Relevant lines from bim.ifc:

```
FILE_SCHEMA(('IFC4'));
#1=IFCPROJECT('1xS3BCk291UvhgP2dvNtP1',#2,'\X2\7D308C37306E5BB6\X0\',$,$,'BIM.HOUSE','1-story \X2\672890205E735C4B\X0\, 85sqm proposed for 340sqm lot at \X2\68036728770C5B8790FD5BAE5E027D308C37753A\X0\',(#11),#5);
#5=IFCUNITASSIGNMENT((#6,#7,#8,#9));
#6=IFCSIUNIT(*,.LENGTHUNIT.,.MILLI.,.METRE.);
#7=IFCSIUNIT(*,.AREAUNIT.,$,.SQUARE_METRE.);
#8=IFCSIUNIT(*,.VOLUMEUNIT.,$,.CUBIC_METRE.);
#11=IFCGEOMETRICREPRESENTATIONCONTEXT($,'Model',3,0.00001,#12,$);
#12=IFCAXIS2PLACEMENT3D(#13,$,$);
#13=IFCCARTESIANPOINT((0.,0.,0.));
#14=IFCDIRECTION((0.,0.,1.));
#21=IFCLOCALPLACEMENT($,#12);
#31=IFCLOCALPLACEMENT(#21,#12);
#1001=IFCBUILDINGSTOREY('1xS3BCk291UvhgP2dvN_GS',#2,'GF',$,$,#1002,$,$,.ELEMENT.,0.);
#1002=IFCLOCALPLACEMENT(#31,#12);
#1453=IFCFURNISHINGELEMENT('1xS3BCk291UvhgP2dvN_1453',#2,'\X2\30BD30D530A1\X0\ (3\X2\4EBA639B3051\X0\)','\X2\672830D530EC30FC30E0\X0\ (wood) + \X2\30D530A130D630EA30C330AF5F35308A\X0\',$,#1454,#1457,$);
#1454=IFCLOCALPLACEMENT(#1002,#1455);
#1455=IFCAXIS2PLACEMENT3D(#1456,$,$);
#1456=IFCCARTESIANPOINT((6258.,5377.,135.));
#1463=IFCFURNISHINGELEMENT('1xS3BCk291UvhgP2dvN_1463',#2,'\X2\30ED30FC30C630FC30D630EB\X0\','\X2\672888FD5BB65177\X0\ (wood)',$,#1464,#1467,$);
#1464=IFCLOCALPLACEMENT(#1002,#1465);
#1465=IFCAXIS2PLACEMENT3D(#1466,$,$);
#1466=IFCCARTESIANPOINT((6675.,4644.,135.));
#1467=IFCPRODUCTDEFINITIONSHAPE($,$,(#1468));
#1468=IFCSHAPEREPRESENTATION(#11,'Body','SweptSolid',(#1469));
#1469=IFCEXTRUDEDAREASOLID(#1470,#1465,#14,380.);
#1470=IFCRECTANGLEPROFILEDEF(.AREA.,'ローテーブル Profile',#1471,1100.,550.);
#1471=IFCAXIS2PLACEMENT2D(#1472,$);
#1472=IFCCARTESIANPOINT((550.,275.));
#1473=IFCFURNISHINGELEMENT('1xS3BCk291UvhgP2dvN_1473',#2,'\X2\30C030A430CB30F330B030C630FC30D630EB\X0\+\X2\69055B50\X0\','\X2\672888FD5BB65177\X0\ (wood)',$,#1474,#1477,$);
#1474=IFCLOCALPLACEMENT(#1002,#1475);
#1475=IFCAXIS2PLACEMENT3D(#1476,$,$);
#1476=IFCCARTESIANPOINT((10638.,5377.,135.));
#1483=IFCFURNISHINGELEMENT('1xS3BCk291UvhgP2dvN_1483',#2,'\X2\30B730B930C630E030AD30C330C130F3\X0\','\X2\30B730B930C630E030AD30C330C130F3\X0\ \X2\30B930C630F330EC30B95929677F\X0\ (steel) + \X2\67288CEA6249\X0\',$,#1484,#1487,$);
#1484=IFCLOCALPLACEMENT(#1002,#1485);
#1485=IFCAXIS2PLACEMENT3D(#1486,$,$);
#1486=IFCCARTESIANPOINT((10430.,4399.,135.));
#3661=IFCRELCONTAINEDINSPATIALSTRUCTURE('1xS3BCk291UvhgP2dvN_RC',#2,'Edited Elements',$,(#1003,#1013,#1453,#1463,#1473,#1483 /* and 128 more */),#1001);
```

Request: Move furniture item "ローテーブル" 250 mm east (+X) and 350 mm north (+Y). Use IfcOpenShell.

```python
import ifcopenshell
import ifcopenshell.api.geometry
import ifcopenshell.util.placement

model = ifcopenshell.open("bim.ifc")

item = model.by_id(1463)
matrix = ifcopenshell.util.placement.get_local_placement(item.ObjectPlacement)
matrix[0, 3] += 250.0
matrix[1, 3] += 350.0
ifcopenshell.api.geometry.edit_object_placement(model, product=item, matrix=matrix, is_si=False)

print(ifcopenshell.util.placement.get_local_placement(item.ObjectPlacement).round(3) + 0.0)

model.write("bim_v2.ifc")
```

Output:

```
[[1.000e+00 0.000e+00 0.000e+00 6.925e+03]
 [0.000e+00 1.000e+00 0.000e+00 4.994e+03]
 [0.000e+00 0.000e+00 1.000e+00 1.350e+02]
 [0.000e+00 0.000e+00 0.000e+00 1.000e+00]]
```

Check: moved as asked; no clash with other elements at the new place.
